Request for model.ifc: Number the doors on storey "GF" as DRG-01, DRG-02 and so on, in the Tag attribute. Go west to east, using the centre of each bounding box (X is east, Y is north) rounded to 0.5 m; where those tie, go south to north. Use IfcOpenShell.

First a look at what the model holds.

```python
import ifcopenshell
import ifcopenshell.util.element
import ifcopenshell.util.placement

model = ifcopenshell.open("model.ifc")
print(model.schema)
storey = next(s for s in model.by_type("IfcBuildingStorey") if s.Name == "GF")
doors = [e for e in ifcopenshell.util.element.get_decomposition(storey) if e.is_a("IfcDoor")]
for e in sorted(doors, key=lambda e: e.id()):
    origin = ifcopenshell.util.placement.get_local_placement(e.ObjectPlacement)[:3, 3]
    print(e.id(), e.Tag, e.Name, origin.round(2) + 0.0, sep=" | ")
```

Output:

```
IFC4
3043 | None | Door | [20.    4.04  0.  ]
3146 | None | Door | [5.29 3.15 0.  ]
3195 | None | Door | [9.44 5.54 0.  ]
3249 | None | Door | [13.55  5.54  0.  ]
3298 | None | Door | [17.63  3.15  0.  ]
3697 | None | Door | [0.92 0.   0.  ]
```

```python
import ifcopenshell
import ifcopenshell.geom
import ifcopenshell.util.element
import ifcopenshell.util.shape

model = ifcopenshell.open("model.ifc")
settings = ifcopenshell.geom.settings()
settings.set("use-world-coords", True)


def centre(element):
    shape = ifcopenshell.geom.create_shape(settings, element)
    return ifcopenshell.util.shape.get_bbox_centroid(shape.geometry)


storey = next(s for s in model.by_type("IfcBuildingStorey") if s.Name == "GF")
doors = [e for e in ifcopenshell.util.element.get_decomposition(storey) if e.is_a("IfcDoor")]

# Insertion points can sit at a corner or the storey origin, so sort by the geometry (in metres).
centres = {e: centre(e) for e in doors}
doors.sort(key=lambda e: (round(centres[e][0] / 0.5), centres[e][1]))

for i, e in enumerate(doors, start=1):
    number = f"DRG-{i:02d}"
    e.Tag = number
    print(e.id(), number)

model.write("model_v2.ifc")
```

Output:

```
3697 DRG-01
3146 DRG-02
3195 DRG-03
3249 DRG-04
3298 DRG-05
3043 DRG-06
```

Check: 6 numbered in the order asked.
